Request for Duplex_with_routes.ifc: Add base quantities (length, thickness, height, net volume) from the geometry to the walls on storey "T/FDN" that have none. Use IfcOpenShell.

First a look at what the model holds.

```python
import ifcopenshell
import ifcopenshell.util.element
import ifcopenshell.util.unit

model = ifcopenshell.open("Duplex_with_routes.ifc")
print(model.schema)
for unit_type in ("LENGTHUNIT", "AREAUNIT", "VOLUMEUNIT"):
    print(unit_type, ifcopenshell.util.unit.calculate_unit_scale(model, unit_type))
storey = next(s for s in model.by_type("IfcBuildingStorey") if s.Name == "T/FDN")
walls = [e for e in ifcopenshell.util.element.get_decomposition(storey) if e.is_a("IfcWall")]
for e in sorted(walls, key=lambda e: e.id()):
    print(e.id(), e.is_a(), e.Name, list(ifcopenshell.util.element.get_psets(e, qtos_only=True)), sep=" | ")
```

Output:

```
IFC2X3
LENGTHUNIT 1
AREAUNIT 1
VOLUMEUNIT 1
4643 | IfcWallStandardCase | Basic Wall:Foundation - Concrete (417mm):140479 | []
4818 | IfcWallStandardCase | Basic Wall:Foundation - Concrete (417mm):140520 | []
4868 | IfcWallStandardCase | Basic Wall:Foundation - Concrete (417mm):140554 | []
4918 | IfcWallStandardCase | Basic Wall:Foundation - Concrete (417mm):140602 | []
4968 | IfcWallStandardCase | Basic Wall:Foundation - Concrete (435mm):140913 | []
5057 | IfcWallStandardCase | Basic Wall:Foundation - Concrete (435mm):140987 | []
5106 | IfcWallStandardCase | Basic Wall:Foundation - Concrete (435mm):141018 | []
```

```python
import ifcopenshell
import ifcopenshell.api.pset
import ifcopenshell.geom
import ifcopenshell.util.element
import ifcopenshell.util.shape
import ifcopenshell.util.unit

model = ifcopenshell.open("Duplex_with_routes.ifc")
unit_scale = ifcopenshell.util.unit.calculate_unit_scale(model)
volume_scale = ifcopenshell.util.unit.calculate_unit_scale(model, "VOLUMEUNIT")
settings = ifcopenshell.geom.settings()

storey = next(s for s in model.by_type("IfcBuildingStorey") if s.Name == "T/FDN")
walls = [e for e in ifcopenshell.util.element.get_decomposition(storey) if e.is_a("IfcWall")]

for e in sorted(walls, key=lambda e: e.id()):
    if ifcopenshell.util.element.get_psets(e, qtos_only=True, should_inherit=False):
        continue
    # Geometry comes back in metres, in the element's own axes.
    shape = ifcopenshell.geom.create_shape(settings, e)
    values = {
        "Length": ifcopenshell.util.shape.get_x(shape.geometry) / unit_scale,
        "Width": ifcopenshell.util.shape.get_y(shape.geometry) / unit_scale,
        "Height": ifcopenshell.util.shape.get_z(shape.geometry) / unit_scale,
        "NetVolume": ifcopenshell.util.shape.get_volume(shape.geometry) / volume_scale,
    }
    qto = ifcopenshell.api.pset.add_qto(model, product=e, name="BaseQuantities")
    ifcopenshell.api.pset.edit_qto(model, qto=qto, properties=values)
    print(e.id(), {k: round(v, 3) for k, v in values.items()})

model.write("Duplex_with_routes_rev.ifc")
```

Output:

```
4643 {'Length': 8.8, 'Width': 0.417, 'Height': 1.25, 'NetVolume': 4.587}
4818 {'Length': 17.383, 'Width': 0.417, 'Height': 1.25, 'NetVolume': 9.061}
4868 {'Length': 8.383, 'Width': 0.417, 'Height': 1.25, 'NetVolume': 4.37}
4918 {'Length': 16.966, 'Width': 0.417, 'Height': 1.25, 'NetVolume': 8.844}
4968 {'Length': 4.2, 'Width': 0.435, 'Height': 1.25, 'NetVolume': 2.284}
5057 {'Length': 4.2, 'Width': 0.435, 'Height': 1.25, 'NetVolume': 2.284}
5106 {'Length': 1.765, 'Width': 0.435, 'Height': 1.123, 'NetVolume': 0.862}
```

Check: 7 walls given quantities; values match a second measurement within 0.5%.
